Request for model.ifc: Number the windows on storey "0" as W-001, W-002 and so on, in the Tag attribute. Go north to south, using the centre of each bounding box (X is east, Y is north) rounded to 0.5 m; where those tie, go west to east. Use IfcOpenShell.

First a look at what the model holds.

```python
import ifcopenshell
import ifcopenshell.util.element
import ifcopenshell.util.placement

model = ifcopenshell.open("model.ifc")
print(model.schema)
storey = next(s for s in model.by_type("IfcBuildingStorey") if s.Name == "0")
windows = [e for e in ifcopenshell.util.element.get_decomposition(storey) if e.is_a("IfcWindow")]
for e in sorted(windows, key=lambda e: e.id()):
    origin = ifcopenshell.util.placement.get_local_placement(e.ObjectPlacement)[:3, 3]
    print(e.id(), e.Tag, e.Name, origin.round(2) + 0.0, sep=" | ")
```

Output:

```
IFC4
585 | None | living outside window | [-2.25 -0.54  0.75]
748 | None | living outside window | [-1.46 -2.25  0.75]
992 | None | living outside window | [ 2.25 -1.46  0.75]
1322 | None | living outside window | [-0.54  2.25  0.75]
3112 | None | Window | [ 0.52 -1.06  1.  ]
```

```python
import ifcopenshell
import ifcopenshell.geom
import ifcopenshell.util.element
import ifcopenshell.util.shape

model = ifcopenshell.open("model.ifc")
settings = ifcopenshell.geom.settings()
settings.set("use-world-coords", True)


def centre(element):
    shape = ifcopenshell.geom.create_shape(settings, element)
    return ifcopenshell.util.shape.get_bbox_centroid(shape.geometry)


storey = next(s for s in model.by_type("IfcBuildingStorey") if s.Name == "0")
windows = [e for e in ifcopenshell.util.element.get_decomposition(storey) if e.is_a("IfcWindow")]

# Insertion points can sit at a corner or the storey origin, so sort by the geometry (in metres).
centres = {e: centre(e) for e in windows}
windows.sort(key=lambda e: (-round(centres[e][1] / 0.5), centres[e][0]))

for i, e in enumerate(windows, start=1):
    number = f"W-0{i:02d}"
    e.Tag = number
    print(e.id(), number)

model.write("model_rev.ifc")
```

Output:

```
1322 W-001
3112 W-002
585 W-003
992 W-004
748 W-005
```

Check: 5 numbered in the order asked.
